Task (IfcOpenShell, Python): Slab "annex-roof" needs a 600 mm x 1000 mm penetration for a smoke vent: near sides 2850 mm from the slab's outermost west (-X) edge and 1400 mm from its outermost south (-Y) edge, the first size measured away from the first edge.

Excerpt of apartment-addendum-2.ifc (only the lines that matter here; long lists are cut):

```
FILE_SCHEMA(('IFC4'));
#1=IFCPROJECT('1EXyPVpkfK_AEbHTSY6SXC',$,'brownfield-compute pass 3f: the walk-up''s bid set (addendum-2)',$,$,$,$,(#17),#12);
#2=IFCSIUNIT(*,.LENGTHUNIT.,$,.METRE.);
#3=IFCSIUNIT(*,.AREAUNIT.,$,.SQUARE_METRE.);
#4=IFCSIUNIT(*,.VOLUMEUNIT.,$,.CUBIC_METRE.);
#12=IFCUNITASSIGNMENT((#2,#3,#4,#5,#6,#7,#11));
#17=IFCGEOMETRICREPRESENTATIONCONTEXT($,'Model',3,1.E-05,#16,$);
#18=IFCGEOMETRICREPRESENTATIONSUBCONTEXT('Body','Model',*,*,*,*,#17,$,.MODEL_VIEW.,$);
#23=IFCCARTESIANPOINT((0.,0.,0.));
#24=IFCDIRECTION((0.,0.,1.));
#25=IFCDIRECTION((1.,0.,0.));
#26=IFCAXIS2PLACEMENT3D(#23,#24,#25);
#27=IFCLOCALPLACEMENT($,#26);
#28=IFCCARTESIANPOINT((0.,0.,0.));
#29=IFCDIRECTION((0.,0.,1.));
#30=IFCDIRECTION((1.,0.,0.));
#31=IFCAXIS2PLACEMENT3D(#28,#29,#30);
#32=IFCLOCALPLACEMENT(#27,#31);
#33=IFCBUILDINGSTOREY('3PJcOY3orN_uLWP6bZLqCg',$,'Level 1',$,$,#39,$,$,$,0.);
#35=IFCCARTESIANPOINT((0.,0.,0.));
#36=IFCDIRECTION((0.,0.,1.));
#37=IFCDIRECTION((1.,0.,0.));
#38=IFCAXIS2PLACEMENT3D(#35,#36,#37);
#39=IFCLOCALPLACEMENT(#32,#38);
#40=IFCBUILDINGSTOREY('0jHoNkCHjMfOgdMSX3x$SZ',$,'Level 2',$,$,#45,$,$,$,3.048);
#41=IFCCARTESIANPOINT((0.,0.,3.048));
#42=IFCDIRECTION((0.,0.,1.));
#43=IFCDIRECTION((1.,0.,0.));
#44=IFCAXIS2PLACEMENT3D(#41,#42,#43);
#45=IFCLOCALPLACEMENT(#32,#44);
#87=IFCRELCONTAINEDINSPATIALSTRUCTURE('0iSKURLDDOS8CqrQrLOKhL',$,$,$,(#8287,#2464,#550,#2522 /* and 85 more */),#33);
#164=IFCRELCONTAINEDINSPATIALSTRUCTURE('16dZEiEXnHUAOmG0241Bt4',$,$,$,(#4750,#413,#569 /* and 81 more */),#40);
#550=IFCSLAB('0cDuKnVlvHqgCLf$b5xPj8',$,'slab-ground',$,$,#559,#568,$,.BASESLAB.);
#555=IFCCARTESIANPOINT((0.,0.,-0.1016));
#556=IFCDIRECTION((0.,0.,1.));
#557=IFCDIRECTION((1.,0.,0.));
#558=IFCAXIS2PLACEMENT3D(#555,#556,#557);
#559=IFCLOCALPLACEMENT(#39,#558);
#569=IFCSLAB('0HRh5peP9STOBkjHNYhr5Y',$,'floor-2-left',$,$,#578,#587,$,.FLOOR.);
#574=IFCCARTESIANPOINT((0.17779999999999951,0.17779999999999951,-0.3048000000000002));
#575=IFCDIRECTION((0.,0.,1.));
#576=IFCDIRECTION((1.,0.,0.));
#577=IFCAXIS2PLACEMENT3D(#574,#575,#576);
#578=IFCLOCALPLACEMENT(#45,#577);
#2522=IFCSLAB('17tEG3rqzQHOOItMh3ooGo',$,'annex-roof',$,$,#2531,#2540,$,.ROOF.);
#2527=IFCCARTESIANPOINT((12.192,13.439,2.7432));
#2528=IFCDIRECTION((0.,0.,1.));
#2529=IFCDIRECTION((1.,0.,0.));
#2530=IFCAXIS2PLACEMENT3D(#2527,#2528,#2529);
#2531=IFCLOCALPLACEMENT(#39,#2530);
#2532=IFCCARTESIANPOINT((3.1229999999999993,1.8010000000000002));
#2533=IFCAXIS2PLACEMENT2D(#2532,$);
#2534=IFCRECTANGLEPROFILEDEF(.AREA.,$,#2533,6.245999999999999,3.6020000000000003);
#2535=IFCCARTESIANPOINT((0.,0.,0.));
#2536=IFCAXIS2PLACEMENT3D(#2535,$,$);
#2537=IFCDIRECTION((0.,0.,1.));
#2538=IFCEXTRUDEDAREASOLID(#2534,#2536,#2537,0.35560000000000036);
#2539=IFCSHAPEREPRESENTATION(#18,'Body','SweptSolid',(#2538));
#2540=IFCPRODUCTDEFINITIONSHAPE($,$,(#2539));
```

```python
import numpy as np
import ifcopenshell
import ifcopenshell.api.feature
import ifcopenshell.api.geometry
import ifcopenshell.api.root
import ifcopenshell.geom
import ifcopenshell.util.placement
import ifcopenshell.util.representation
import ifcopenshell.util.shape
import ifcopenshell.util.unit

model = ifcopenshell.open("apartment-addendum-2.ifc")
unit_scale = ifcopenshell.util.unit.calculate_unit_scale(model)
settings = ifcopenshell.geom.settings()


def volume(element):
    """Net volume in cubic metres, openings subtracted."""
    shape = ifcopenshell.geom.create_shape(settings, element)
    return ifcopenshell.util.shape.get_volume(shape.geometry)


slab = model.by_id(2522)
before = volume(slab)

# Extent in the slab's own axes, in metres. The edges named are its -X and -Y sides.
slab_shape = ifcopenshell.geom.create_shape(settings, slab)
vertices = ifcopenshell.util.shape.get_vertices(slab_shape.geometry)
x_min, y_min, bottom = vertices.min(axis=0)
top = vertices[:, 2].max()

opening = ifcopenshell.api.root.create_entity(model, ifc_class="IfcOpeningElement", name="Smoke vent opening", predefined_type="OPENING")
context = ifcopenshell.util.representation.get_context(model, "Model", "Body", "MODEL_VIEW")
width, depth = 0.6, 1
outline = [(0.0, 0.0), (width, 0.0), (width, depth), (0.0, depth), (0.0, 0.0)]
# Overshoot both faces by 50 mm so the cut is clean.
shape = ifcopenshell.api.geometry.add_slab_representation(
    model, context=context, depth=top - bottom + 0.1, polyline=outline
)
ifcopenshell.api.geometry.assign_representation(model, product=opening, representation=shape)

matrix = ifcopenshell.util.placement.get_local_placement(slab.ObjectPlacement)
matrix[:, 3] = matrix @ np.append(np.array([x_min + 2.85, y_min + 1.4, bottom - 0.05]) / unit_scale, 1.0)
ifcopenshell.api.geometry.edit_object_placement(model, product=opening, matrix=matrix, is_si=False)
ifcopenshell.api.feature.add_feature(model, feature=opening, element=slab)

after = volume(slab)

print(f"slab volume {before:.3f} -> {after:.3f} m3")

model.write("apartment-addendum-2_rev.ifc")
```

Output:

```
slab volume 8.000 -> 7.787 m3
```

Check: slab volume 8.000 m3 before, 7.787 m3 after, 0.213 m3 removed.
